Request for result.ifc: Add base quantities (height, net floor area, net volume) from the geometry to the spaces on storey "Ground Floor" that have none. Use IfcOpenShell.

First a look at what the model holds.

```python
import ifcopenshell
import ifcopenshell.util.element
import ifcopenshell.util.unit

model = ifcopenshell.open("result.ifc")
print(model.schema)
for unit_type in ("LENGTHUNIT", "AREAUNIT", "VOLUMEUNIT"):
    print(unit_type, ifcopenshell.util.unit.calculate_unit_scale(model, unit_type))
storey = next(s for s in model.by_type("IfcBuildingStorey") if s.Name == "Ground Floor")
spaces = [e for e in ifcopenshell.util.element.get_decomposition(storey) if e.is_a("IfcSpace")]
for e in sorted(spaces, key=lambda e: e.id()):
    print(e.id(), e.is_a(), e.Name, list(ifcopenshell.util.element.get_psets(e, qtos_only=True)), sep=" | ")
```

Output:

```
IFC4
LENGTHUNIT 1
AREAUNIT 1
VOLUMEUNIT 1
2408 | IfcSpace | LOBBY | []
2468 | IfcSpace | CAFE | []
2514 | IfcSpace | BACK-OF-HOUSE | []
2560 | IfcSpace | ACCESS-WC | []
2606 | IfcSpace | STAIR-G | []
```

```python
import ifcopenshell
import ifcopenshell.api.pset
import ifcopenshell.geom
import ifcopenshell.util.element
import ifcopenshell.util.shape
import ifcopenshell.util.unit

model = ifcopenshell.open("result.ifc")
unit_scale = ifcopenshell.util.unit.calculate_unit_scale(model)
area_scale = ifcopenshell.util.unit.calculate_unit_scale(model, "AREAUNIT")
volume_scale = ifcopenshell.util.unit.calculate_unit_scale(model, "VOLUMEUNIT")
settings = ifcopenshell.geom.settings()

storey = next(s for s in model.by_type("IfcBuildingStorey") if s.Name == "Ground Floor")
spaces = [e for e in ifcopenshell.util.element.get_decomposition(storey) if e.is_a("IfcSpace")]

for e in sorted(spaces, key=lambda e: e.id()):
    if ifcopenshell.util.element.get_psets(e, qtos_only=True, should_inherit=False):
        continue
    # Geometry comes back in metres, in the element's own axes.
    shape = ifcopenshell.geom.create_shape(settings, e)
    values = {
        "Height": ifcopenshell.util.shape.get_z(shape.geometry) / unit_scale,
        "NetFloorArea": ifcopenshell.util.shape.get_footprint_area(shape.geometry) / area_scale,
        "NetVolume": ifcopenshell.util.shape.get_volume(shape.geometry) / volume_scale,
    }
    qto = ifcopenshell.api.pset.add_qto(model, product=e, name="Qto_SpaceBaseQuantities")
    ifcopenshell.api.pset.edit_qto(model, qto=qto, properties=values)
    print(e.id(), {k: round(v, 3) for k, v in values.items()})

model.write("result_edited.ifc")
```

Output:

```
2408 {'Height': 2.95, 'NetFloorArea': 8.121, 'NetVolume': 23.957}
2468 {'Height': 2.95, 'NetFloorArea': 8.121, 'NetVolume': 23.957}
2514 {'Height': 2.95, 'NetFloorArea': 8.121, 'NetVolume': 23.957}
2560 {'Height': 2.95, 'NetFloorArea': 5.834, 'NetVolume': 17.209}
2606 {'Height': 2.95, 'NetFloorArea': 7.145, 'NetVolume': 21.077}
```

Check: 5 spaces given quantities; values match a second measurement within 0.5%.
